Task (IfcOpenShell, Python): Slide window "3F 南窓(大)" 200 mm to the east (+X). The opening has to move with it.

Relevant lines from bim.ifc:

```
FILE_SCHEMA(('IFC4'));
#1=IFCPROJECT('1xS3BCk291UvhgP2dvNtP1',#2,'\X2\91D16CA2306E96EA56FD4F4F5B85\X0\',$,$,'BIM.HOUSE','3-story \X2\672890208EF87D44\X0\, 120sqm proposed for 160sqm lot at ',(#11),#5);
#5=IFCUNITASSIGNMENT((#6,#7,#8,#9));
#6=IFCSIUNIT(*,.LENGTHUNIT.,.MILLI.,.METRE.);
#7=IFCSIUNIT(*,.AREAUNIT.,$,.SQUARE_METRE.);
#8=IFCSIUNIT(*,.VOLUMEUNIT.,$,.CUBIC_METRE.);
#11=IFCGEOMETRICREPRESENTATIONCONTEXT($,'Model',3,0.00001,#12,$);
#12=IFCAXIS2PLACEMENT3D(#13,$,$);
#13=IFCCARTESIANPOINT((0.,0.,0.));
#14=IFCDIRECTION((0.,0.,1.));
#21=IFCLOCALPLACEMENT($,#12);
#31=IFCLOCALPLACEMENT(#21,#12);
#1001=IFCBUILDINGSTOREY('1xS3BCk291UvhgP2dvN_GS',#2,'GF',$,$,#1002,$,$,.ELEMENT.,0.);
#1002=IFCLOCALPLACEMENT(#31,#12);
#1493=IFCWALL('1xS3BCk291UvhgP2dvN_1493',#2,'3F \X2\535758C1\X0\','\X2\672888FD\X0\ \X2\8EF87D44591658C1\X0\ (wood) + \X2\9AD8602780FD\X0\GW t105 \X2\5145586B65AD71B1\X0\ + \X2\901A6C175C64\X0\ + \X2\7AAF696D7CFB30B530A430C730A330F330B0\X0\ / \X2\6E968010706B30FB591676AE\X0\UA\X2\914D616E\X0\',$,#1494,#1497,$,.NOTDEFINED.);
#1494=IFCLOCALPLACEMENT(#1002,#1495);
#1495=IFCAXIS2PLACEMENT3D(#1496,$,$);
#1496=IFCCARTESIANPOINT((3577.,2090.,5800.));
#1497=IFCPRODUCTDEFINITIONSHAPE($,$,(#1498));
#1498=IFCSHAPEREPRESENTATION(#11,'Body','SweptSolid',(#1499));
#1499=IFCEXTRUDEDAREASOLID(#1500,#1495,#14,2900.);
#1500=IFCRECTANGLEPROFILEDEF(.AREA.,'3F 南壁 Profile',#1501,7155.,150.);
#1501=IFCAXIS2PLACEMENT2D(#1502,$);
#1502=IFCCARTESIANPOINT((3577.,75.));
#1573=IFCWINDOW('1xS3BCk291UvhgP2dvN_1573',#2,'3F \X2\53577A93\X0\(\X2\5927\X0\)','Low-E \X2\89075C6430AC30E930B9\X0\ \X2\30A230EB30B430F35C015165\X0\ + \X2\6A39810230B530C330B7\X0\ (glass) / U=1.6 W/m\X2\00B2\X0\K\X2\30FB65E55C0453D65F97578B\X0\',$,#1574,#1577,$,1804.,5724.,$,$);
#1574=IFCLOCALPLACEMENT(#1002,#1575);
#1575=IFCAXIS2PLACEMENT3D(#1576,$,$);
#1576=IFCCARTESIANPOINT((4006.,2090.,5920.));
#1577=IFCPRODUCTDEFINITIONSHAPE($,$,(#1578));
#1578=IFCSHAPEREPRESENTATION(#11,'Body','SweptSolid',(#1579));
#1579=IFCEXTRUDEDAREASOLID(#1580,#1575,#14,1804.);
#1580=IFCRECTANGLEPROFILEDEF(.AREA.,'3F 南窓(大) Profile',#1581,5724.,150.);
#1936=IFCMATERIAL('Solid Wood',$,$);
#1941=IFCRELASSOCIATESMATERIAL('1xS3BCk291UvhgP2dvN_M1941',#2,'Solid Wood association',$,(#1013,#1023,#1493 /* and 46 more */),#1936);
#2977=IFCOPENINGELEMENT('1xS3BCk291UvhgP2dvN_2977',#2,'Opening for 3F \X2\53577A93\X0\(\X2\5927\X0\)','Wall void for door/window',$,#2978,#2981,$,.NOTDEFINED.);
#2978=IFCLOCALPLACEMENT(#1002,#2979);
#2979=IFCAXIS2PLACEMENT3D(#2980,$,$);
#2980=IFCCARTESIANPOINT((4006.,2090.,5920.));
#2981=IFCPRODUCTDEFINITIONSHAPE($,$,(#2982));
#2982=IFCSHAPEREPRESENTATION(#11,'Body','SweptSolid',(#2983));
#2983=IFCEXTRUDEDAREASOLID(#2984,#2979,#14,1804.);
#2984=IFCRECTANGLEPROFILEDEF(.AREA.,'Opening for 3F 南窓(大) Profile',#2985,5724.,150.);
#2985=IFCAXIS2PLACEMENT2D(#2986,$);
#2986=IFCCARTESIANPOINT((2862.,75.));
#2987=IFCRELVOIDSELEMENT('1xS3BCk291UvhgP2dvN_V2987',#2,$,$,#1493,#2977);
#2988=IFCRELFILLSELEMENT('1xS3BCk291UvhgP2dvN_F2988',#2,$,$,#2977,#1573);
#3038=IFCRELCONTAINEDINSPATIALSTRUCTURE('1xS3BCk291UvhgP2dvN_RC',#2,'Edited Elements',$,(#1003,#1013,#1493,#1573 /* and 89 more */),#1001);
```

```python
import ifcopenshell
import ifcopenshell.api.geometry
import ifcopenshell.util.placement
import ifcopenshell.util.unit

model = ifcopenshell.open("bim.ifc")
unit_scale = ifcopenshell.util.unit.calculate_unit_scale(model)

window = model.by_id(1573)
opening = window.FillsVoids[0].RelatingOpeningElement
wall = opening.VoidsElements[0].RelatingBuildingElement

wall_matrix = ifcopenshell.util.placement.get_local_placement(wall.ObjectPlacement)
shift = wall_matrix[:3, 0] * 0.2 / unit_scale
before = ifcopenshell.util.placement.get_local_placement(window.ObjectPlacement)[:3, 3].copy()

# The window is not placed relative to its opening, so move both.
for product in (opening, window):
    matrix = ifcopenshell.util.placement.get_local_placement(product.ObjectPlacement)
    matrix[:3, 3] += shift
    ifcopenshell.api.geometry.edit_object_placement(model, product=product, matrix=matrix, is_si=False)

after = ifcopenshell.util.placement.get_local_placement(window.ObjectPlacement)[:3, 3]
print("window moved by", (after - before).round(3) + 0.0)

model.write("bim_updated.ifc")
```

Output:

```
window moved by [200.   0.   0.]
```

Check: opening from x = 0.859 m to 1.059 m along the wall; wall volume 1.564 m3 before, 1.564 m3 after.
